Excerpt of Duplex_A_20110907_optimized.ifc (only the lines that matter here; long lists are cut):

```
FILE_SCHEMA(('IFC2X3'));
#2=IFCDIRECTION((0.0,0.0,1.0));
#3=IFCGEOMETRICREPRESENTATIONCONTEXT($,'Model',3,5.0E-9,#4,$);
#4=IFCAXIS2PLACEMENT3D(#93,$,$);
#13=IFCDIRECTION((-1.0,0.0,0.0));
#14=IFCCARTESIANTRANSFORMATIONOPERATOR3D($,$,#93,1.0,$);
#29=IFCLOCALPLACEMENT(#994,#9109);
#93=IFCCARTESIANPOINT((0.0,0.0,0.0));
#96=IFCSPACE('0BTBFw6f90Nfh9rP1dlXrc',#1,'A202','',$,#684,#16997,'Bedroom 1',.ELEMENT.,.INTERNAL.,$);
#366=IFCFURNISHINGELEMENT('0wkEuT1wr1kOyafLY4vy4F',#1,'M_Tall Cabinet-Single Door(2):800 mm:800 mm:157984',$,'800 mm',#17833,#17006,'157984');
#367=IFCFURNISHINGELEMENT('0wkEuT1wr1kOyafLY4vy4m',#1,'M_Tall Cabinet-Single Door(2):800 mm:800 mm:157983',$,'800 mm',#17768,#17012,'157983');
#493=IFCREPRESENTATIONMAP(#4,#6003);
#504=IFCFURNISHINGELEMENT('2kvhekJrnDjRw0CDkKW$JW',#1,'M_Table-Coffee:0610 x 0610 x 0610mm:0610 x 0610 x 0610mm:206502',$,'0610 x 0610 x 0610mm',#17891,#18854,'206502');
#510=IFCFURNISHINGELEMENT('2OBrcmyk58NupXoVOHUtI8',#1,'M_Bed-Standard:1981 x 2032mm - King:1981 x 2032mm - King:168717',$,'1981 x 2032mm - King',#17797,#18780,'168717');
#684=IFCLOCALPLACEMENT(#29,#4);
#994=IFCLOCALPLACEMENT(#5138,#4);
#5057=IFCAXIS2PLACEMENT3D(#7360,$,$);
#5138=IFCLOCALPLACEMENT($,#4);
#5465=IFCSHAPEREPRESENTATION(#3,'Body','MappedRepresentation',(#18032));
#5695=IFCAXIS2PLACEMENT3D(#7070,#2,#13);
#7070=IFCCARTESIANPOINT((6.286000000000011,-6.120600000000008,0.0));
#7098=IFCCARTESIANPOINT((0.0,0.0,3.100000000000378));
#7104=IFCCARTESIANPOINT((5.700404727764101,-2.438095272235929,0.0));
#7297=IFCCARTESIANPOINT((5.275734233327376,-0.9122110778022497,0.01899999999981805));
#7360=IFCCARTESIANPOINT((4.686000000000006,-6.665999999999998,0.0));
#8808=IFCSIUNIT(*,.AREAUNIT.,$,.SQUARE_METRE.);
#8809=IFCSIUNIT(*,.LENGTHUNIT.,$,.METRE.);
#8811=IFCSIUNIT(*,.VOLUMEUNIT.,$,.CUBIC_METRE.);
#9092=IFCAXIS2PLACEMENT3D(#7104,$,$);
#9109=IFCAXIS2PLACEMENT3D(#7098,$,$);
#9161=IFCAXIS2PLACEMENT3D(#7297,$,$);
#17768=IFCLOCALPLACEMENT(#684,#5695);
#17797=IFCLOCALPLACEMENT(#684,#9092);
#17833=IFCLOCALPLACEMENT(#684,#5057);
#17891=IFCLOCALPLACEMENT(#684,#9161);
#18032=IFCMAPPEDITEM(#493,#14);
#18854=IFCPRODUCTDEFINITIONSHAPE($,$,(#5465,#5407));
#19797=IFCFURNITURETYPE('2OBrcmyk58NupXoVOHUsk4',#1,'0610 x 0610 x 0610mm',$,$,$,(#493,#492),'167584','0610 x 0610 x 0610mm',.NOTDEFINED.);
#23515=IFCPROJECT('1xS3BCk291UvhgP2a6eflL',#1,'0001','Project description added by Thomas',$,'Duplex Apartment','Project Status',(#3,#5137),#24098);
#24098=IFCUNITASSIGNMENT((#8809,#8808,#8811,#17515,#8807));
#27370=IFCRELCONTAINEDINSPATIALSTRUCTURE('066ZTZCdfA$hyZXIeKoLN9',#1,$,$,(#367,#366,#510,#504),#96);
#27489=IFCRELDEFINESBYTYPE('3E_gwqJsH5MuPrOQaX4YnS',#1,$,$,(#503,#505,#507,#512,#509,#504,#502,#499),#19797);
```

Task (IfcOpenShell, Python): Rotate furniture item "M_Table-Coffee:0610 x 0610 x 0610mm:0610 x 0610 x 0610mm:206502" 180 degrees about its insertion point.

```python
import ifcopenshell
import ifcopenshell.api.geometry
import ifcopenshell.util.placement

model = ifcopenshell.open("Duplex_A_20110907_optimized.ifc")

item = model.by_id(504)
matrix = ifcopenshell.util.placement.get_local_placement(item.ObjectPlacement)
matrix = matrix @ ifcopenshell.util.placement.rotation(180, "Z")
ifcopenshell.api.geometry.edit_object_placement(model, product=item, matrix=matrix, is_si=False)

print(ifcopenshell.util.placement.get_local_placement(item.ObjectPlacement).round(3) + 0.0)

model.write("Duplex_A_20110907_optimized_v2.ifc")
```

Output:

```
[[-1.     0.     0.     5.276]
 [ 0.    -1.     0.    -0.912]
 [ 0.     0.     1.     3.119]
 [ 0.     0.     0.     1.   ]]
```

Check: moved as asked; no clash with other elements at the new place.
